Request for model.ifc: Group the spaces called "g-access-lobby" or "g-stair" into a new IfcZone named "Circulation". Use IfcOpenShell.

First a look at what the model holds.

```python
import ifcopenshell

model = ifcopenshell.open("model.ifc")
print(model.schema)
seen = {}
for space in model.by_type("IfcSpace"):
    seen[space.LongName] = seen.get(space.LongName, 0) + 1
for name, count in sorted(seen.items(), key=str):
    print(count, "x", name)
print("zones:", [z.Name for z in model.by_type("IfcZone")][:20])
```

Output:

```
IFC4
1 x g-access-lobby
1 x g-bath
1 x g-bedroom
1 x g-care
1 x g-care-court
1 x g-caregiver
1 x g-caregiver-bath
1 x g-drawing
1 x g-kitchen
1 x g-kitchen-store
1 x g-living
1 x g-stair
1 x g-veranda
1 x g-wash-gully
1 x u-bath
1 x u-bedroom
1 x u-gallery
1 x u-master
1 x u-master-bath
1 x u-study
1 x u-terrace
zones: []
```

```python
import ifcopenshell
import ifcopenshell.api.group
import ifcopenshell.api.root

model = ifcopenshell.open("model.ifc")

names = {"g-access-lobby", "g-stair"}
spaces = [s for s in model.by_type("IfcSpace") if s.LongName in names]

zone = ifcopenshell.api.root.create_entity(model, ifc_class="IfcZone", name="Circulation")
ifcopenshell.api.group.assign_group(model, products=spaces, group=zone)
print(len(spaces), "spaces in", zone.Name)

model.write("model_v2.ifc")
```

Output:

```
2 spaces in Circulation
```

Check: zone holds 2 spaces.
